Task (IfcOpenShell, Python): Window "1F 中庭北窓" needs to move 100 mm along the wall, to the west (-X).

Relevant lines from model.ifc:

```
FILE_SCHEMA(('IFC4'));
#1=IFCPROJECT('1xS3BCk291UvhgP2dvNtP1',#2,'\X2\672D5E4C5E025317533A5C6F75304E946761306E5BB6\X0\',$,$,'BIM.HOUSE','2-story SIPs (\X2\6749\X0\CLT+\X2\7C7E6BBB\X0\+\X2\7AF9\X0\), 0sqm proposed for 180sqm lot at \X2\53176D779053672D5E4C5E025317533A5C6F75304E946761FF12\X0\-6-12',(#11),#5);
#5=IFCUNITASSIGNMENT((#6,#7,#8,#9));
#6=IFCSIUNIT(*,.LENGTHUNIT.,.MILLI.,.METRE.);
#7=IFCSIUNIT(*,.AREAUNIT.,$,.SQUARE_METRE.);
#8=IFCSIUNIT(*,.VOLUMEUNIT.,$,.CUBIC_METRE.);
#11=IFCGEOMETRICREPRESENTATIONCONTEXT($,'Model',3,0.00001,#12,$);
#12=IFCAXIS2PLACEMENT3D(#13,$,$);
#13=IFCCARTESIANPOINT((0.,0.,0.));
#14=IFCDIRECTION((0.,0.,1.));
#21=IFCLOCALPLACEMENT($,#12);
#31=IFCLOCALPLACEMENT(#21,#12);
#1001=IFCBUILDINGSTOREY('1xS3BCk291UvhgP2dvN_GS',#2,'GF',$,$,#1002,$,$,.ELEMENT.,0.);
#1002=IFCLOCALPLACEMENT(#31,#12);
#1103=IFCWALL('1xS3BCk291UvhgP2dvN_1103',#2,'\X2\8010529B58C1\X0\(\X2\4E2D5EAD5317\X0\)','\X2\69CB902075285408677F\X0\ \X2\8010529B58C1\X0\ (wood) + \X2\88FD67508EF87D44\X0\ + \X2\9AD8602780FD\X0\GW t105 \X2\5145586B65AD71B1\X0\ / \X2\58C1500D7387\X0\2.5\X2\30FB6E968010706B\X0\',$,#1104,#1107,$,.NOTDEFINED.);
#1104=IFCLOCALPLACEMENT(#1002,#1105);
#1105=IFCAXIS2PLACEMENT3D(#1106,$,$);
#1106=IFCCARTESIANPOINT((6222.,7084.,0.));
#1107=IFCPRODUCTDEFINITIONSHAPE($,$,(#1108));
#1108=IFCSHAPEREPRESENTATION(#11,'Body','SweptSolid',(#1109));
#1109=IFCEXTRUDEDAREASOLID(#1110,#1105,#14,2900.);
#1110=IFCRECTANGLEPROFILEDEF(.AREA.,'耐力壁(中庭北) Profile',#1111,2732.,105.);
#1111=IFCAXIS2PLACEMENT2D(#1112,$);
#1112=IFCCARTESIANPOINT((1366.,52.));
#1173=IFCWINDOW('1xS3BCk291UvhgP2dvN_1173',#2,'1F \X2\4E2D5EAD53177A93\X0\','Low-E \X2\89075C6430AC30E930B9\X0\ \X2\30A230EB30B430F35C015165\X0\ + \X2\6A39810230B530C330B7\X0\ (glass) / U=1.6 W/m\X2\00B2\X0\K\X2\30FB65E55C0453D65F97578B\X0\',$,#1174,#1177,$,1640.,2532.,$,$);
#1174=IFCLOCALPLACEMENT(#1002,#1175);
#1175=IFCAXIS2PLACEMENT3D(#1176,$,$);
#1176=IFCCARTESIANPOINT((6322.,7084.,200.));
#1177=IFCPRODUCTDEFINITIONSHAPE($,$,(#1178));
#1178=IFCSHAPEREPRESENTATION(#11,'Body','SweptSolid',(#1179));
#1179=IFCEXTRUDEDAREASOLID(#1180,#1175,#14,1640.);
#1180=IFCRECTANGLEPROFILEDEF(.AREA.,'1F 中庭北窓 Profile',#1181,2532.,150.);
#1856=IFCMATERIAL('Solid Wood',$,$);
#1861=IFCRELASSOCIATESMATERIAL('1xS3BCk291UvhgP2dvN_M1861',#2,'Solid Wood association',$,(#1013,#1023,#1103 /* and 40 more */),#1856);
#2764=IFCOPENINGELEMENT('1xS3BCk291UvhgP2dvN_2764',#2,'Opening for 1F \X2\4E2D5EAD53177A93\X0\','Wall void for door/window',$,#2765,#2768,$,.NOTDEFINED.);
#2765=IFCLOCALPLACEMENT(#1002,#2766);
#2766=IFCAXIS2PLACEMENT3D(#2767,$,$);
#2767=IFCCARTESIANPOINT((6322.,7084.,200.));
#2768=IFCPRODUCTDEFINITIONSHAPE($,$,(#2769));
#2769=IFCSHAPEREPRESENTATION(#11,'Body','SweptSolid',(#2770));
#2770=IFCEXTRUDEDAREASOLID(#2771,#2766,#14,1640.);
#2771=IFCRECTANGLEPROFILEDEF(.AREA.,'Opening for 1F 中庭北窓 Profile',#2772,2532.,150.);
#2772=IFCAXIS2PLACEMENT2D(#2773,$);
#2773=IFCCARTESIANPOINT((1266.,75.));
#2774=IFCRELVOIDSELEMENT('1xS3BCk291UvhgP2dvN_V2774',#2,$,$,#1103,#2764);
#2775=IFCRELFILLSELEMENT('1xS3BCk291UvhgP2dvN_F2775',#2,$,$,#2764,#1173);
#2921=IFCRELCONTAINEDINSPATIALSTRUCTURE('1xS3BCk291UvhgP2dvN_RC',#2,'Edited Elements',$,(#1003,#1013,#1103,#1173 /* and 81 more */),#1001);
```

```python
import ifcopenshell
import ifcopenshell.api.geometry
import ifcopenshell.util.placement

model = ifcopenshell.open("model.ifc")

window = model.by_guid("1xS3BCk291UvhgP2dvN_1173")
opening = window.FillsVoids[0].RelatingOpeningElement
wall = opening.VoidsElements[0].RelatingBuildingElement

wall_matrix = ifcopenshell.util.placement.get_local_placement(wall.ObjectPlacement)
shift = wall_matrix[:3, 0] * -100.0
before = ifcopenshell.util.placement.get_local_placement(window.ObjectPlacement)[:3, 3].copy()

# The window is not placed relative to its opening, so move both.
for product in (opening, window):
    matrix = ifcopenshell.util.placement.get_local_placement(product.ObjectPlacement)
    matrix[:3, 3] += shift
    ifcopenshell.api.geometry.edit_object_placement(model, product=product, matrix=matrix, is_si=False)

after = ifcopenshell.util.placement.get_local_placement(window.ObjectPlacement)[:3, 3]
print("window moved by", (after - before).round(3) + 0.0)

model.write("model-out.ifc")
```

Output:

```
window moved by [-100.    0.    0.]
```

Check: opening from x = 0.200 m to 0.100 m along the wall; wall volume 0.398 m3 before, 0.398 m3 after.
